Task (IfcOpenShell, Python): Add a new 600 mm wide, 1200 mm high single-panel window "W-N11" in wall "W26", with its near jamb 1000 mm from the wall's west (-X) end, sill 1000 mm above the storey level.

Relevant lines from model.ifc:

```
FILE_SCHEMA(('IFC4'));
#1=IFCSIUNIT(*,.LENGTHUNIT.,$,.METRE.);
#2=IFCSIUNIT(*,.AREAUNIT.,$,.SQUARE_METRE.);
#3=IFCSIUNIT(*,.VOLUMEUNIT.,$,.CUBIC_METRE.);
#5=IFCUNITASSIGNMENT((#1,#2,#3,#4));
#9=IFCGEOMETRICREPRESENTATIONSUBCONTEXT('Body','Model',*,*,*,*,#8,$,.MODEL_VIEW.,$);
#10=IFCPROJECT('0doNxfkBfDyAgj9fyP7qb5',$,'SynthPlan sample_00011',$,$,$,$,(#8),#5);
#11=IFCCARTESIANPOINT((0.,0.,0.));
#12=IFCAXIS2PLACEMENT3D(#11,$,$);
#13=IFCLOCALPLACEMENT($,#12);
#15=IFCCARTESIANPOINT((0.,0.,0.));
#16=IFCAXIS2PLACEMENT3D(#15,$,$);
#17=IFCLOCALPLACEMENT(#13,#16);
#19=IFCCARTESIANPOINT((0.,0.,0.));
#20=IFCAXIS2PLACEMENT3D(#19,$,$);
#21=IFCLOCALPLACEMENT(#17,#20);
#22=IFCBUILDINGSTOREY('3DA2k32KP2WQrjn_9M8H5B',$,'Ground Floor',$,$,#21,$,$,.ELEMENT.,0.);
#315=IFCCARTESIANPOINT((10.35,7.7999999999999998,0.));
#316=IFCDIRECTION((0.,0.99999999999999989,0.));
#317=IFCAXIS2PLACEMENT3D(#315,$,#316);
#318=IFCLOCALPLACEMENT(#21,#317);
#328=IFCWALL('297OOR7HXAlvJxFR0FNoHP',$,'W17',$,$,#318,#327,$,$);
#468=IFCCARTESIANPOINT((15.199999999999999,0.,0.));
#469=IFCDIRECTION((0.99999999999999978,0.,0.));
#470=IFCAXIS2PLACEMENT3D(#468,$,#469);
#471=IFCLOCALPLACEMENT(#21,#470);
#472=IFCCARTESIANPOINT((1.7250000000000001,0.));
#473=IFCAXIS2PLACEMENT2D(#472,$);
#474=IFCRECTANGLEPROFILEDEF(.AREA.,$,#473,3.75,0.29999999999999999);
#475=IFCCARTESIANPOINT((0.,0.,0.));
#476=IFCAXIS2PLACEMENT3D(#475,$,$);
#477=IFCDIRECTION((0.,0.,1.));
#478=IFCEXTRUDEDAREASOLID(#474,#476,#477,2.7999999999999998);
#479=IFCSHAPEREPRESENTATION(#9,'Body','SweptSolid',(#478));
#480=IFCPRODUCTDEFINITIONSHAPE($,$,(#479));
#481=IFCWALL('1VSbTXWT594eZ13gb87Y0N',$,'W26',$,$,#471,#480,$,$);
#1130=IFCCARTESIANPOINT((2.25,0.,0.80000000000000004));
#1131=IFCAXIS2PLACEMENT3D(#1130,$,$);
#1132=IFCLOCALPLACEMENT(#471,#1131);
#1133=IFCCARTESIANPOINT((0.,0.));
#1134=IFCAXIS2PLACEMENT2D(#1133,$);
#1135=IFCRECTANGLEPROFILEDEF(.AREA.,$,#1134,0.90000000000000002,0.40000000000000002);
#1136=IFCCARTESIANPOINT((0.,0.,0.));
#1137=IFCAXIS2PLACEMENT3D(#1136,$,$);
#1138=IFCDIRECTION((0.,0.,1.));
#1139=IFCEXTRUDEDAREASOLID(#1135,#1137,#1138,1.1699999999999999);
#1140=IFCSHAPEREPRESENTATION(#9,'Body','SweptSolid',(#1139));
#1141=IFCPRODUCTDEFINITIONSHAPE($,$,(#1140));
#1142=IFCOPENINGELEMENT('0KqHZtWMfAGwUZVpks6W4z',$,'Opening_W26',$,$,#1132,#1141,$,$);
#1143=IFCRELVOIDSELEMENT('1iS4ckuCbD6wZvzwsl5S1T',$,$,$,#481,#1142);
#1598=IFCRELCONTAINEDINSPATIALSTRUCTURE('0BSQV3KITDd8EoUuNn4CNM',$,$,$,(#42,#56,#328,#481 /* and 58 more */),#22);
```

```python
import numpy as np
import ifcopenshell
import ifcopenshell.api.feature
import ifcopenshell.api.geometry
import ifcopenshell.api.root
import ifcopenshell.api.spatial
import ifcopenshell.geom
import ifcopenshell.util.element
import ifcopenshell.util.placement
import ifcopenshell.util.representation
import ifcopenshell.util.shape
import ifcopenshell.util.unit

model = ifcopenshell.open("model.ifc")
unit_scale = ifcopenshell.util.unit.calculate_unit_scale(model)
settings = ifcopenshell.geom.settings()


def volume(element):
    """Net volume in cubic metres, openings subtracted."""
    shape = ifcopenshell.geom.create_shape(settings, element)
    return ifcopenshell.util.shape.get_volume(shape.geometry)


wall = model.by_guid("1VSbTXWT594eZ13gb87Y0N")
storey = ifcopenshell.util.element.get_container(wall, ifc_class="IfcBuildingStorey")
context = ifcopenshell.util.representation.get_context(model, "Model", "Body", "MODEL_VIEW")
before = volume(wall)

width, height, from_end, sill = 0.6, 1.2, 1, 1  # metres

# The wall runs along its own X axis, and the end named is its -X end.
wall_shape = ifcopenshell.geom.create_shape(settings, wall)
x, y, z = ifcopenshell.util.shape.get_vertices(wall_shape.geometry).T
start = x.min() + from_end
face, thickness = float(y.min()), float(y.max() - y.min())
wall_matrix = ifcopenshell.util.placement.get_local_placement(wall.ObjectPlacement)
level = ifcopenshell.util.placement.get_local_placement(storey.ObjectPlacement)[2, 3]


def in_wall(x, y):
    """Placement at x, y metres in the wall's axes, at sill height."""
    matrix = wall_matrix.copy()
    matrix[:, 3] = wall_matrix @ np.array([x / unit_scale, y / unit_scale, 0.0, 1.0])
    matrix[2, 3] = level + sill / unit_scale
    return matrix


# Opening: a box that overshoots both wall faces by 50 mm.
opening = ifcopenshell.api.root.create_entity(model, ifc_class="IfcOpeningElement", predefined_type="OPENING")
box = ifcopenshell.api.geometry.add_wall_representation(
    model, context=context, length=width, height=height, thickness=thickness + 0.1
)
ifcopenshell.api.geometry.assign_representation(model, product=opening, representation=box)
ifcopenshell.api.geometry.edit_object_placement(model, product=opening, matrix=in_wall(start, face - 0.05), is_si=False)
ifcopenshell.api.feature.add_feature(model, feature=opening, element=wall)

window = ifcopenshell.api.root.create_entity(model, ifc_class="IfcWindow", name="W-N11", predefined_type="WINDOW")
window.OverallWidth, window.OverallHeight = width / unit_scale, height / unit_scale
window.PartitioningType = "SINGLE_PANEL"
body = ifcopenshell.api.geometry.add_window_representation(
    model,
    context=context,
    overall_width=window.OverallWidth,
    overall_height=window.OverallHeight,
    partition_type="SINGLE_PANEL",
)
ifcopenshell.api.geometry.assign_representation(model, product=window, representation=body)
ifcopenshell.api.spatial.assign_container(model, products=[window], relating_structure=storey)
ifcopenshell.api.feature.add_filling(model, opening=opening, element=window)

# Centre the window in the wall's thickness.
ifcopenshell.api.geometry.edit_object_placement(model, product=window, matrix=in_wall(start, face), is_si=False)
window_shape = ifcopenshell.geom.create_shape(settings, window)
depth = ifcopenshell.util.shape.get_vertices(window_shape.geometry)[:, 1]
offset = face + thickness / 2 - (depth.min() + depth.max()) / 2
ifcopenshell.api.geometry.edit_object_placement(model, product=window, matrix=in_wall(start, offset), is_si=False)

after = volume(wall)

print(f"wall volume {before:.3f} -> {after:.3f} m3")

model.write("model-out.ifc")
```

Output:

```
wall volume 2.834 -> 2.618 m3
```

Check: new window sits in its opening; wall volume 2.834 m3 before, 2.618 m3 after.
